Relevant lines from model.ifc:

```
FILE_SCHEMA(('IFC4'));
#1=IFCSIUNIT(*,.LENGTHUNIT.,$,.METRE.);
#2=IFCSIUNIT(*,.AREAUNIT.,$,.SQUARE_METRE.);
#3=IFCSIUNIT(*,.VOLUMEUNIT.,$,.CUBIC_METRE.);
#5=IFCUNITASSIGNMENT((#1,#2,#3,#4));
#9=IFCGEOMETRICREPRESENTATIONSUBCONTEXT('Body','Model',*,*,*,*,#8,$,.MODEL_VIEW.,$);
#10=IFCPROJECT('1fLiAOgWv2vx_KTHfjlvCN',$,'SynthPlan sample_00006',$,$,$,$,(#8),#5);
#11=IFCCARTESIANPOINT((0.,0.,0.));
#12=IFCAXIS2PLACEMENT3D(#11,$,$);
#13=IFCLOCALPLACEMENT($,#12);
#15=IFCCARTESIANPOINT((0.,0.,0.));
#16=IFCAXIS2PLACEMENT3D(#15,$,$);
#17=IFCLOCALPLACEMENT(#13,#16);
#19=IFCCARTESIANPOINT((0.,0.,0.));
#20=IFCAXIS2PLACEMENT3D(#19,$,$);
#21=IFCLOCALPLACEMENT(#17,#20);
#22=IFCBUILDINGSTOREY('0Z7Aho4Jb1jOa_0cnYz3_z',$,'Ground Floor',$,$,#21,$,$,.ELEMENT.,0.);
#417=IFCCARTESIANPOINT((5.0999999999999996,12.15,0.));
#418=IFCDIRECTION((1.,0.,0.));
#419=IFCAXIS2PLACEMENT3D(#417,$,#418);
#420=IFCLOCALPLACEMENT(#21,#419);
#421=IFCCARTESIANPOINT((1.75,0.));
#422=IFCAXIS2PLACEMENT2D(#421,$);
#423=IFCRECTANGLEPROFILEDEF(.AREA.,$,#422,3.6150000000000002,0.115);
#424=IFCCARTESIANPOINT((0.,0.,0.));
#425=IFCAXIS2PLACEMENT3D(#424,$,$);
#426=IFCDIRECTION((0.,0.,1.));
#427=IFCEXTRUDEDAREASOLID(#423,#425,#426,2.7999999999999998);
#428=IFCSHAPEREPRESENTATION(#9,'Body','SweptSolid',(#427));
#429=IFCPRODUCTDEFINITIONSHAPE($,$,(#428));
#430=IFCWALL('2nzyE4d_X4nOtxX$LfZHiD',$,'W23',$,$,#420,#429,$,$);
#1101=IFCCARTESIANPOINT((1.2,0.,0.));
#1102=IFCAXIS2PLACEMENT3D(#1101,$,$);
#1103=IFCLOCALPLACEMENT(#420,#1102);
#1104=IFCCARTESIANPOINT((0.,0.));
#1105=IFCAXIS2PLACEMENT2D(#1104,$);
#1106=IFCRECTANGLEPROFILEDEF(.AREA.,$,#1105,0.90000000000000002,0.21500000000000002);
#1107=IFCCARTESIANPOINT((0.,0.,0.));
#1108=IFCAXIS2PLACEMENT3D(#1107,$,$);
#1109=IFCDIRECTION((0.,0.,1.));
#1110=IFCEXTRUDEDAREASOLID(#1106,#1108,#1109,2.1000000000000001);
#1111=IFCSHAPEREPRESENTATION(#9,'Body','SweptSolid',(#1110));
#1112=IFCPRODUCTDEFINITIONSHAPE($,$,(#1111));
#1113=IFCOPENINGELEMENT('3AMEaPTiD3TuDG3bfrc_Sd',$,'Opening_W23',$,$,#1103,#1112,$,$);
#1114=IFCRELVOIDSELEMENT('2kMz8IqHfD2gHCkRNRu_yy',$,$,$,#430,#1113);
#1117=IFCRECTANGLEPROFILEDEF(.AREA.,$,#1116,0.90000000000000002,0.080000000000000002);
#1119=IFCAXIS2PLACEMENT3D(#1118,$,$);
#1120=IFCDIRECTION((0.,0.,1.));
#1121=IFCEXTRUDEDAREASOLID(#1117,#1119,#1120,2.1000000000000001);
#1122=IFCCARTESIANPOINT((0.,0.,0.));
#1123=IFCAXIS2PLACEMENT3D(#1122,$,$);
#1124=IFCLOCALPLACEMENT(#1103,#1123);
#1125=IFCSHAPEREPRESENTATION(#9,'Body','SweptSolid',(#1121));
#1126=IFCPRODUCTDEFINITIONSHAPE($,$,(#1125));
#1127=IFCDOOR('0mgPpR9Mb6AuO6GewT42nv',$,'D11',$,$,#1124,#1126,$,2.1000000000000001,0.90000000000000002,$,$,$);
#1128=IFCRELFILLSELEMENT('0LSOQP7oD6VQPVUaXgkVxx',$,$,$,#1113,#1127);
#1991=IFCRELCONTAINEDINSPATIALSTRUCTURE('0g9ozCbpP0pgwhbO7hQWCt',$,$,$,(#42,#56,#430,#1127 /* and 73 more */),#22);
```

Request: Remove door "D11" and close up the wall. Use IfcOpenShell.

```python
import ifcopenshell
import ifcopenshell.api.feature
import ifcopenshell.api.root
import ifcopenshell.geom
import ifcopenshell.util.shape

model = ifcopenshell.open("model.ifc")
settings = ifcopenshell.geom.settings()


def volume(element):
    """Net volume in cubic metres, openings subtracted."""
    shape = ifcopenshell.geom.create_shape(settings, element)
    return ifcopenshell.util.shape.get_volume(shape.geometry)


door = model.by_id(1127)
opening = door.FillsVoids[0].RelatingOpeningElement
wall = opening.VoidsElements[0].RelatingBuildingElement
before = volume(wall)

ifcopenshell.api.root.remove_product(model, product=door)
ifcopenshell.api.feature.remove_feature(model, feature=opening)

after = volume(wall)

print(f"wall volume {before:.3f} -> {after:.3f} m3")

model.write("model_rev.ifc")
```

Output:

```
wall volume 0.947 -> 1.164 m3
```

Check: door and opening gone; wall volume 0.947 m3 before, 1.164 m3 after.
